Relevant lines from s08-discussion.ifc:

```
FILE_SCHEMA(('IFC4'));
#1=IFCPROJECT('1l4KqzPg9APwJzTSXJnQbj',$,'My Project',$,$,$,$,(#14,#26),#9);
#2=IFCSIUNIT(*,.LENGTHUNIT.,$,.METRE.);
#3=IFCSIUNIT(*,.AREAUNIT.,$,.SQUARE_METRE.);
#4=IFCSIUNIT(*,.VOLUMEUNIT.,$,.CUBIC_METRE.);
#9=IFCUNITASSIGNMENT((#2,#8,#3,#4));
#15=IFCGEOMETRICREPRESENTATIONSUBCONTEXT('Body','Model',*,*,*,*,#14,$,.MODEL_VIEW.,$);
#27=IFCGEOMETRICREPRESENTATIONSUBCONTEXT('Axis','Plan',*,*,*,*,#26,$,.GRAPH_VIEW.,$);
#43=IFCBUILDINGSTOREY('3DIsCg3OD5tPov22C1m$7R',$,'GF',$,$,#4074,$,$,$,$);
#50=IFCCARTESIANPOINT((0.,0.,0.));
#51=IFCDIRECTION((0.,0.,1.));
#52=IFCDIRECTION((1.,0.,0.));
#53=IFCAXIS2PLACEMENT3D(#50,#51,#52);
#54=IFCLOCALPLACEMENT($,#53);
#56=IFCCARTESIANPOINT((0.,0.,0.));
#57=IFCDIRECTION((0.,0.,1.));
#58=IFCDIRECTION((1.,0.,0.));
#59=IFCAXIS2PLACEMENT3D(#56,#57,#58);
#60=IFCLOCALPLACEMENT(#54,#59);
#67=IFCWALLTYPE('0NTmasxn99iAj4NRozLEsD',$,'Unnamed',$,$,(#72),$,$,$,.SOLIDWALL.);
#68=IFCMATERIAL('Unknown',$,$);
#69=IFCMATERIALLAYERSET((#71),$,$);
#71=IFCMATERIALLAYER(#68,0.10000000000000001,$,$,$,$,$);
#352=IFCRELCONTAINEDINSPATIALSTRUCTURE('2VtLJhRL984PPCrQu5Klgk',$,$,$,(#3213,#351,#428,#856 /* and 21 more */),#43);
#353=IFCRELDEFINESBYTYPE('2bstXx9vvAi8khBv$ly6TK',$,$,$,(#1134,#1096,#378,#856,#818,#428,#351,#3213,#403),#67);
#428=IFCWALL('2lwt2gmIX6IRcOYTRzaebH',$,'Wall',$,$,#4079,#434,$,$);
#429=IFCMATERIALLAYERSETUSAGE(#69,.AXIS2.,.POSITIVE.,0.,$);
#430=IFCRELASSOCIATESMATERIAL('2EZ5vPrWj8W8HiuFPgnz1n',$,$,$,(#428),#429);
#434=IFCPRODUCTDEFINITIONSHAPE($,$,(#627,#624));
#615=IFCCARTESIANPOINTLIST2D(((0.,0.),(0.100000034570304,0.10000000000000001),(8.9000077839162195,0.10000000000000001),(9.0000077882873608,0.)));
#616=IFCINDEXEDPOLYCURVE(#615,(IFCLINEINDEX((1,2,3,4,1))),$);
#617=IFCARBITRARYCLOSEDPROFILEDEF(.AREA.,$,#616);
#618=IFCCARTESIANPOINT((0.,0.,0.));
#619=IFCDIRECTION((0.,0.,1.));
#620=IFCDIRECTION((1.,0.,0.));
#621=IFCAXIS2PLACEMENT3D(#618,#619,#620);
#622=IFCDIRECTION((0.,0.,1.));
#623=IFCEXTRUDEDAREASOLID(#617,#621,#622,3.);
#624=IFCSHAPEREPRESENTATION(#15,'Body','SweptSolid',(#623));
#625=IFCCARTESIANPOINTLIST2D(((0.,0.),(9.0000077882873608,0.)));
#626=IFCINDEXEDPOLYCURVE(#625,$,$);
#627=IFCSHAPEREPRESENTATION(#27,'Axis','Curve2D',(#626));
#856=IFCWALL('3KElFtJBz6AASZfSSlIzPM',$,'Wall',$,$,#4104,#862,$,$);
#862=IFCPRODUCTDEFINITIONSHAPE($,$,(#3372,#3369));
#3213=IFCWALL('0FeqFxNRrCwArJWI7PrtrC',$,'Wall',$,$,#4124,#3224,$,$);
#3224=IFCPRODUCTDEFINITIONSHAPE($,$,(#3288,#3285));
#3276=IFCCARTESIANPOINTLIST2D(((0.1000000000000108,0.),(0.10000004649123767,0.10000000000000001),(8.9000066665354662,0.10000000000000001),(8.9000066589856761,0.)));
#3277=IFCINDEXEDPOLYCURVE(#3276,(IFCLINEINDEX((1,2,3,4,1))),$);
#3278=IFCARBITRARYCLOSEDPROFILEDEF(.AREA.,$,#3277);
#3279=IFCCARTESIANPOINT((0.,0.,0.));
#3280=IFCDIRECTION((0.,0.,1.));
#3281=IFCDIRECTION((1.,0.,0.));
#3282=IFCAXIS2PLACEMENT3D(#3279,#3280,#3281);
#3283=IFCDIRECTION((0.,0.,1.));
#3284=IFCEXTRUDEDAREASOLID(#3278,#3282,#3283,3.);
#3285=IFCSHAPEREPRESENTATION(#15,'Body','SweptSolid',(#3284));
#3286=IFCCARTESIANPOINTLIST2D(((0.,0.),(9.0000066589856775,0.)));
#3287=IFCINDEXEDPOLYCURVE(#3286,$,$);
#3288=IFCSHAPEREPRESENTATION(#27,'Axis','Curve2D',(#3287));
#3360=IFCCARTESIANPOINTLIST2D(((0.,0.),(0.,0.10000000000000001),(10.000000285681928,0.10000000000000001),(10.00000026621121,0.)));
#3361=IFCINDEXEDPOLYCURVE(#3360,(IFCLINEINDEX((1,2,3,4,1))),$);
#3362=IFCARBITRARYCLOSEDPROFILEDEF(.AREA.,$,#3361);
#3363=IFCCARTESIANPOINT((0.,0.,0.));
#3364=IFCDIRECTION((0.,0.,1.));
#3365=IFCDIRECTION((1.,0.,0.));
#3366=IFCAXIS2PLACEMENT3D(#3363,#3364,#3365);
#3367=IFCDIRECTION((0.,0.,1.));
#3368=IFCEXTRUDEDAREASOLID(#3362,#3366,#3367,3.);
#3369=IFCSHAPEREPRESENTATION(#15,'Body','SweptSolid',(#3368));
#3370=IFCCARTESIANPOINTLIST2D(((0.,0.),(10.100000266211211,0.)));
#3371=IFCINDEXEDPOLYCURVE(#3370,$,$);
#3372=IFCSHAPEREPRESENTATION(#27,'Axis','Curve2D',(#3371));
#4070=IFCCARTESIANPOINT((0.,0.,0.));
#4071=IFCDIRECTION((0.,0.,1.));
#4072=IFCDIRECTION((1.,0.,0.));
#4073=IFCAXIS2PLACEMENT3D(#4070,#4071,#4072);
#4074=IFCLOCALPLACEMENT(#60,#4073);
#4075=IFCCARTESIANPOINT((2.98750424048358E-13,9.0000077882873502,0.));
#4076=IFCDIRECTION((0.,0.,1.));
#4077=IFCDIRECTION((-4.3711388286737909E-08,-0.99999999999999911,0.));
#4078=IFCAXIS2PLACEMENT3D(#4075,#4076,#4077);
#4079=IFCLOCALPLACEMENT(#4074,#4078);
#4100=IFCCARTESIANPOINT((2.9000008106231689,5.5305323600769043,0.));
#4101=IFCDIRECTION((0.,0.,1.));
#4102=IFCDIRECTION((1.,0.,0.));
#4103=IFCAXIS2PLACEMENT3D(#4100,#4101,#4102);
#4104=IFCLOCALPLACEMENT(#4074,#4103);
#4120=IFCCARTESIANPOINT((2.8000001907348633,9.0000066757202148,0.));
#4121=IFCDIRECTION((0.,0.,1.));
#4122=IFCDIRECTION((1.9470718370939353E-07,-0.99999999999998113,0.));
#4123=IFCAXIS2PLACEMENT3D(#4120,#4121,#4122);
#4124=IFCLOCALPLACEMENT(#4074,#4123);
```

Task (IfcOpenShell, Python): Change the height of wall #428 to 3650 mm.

```python
import ifcopenshell
import ifcopenshell.geom
import ifcopenshell.util.representation
import ifcopenshell.util.shape
import ifcopenshell.util.unit

model = ifcopenshell.open("s08-discussion.ifc")
unit_scale = ifcopenshell.util.unit.calculate_unit_scale(model)
settings = ifcopenshell.geom.settings()


def volume(element):
    """Net volume in cubic metres, openings subtracted."""
    shape = ifcopenshell.geom.create_shape(settings, element)
    return ifcopenshell.util.shape.get_volume(shape.geometry)


wall = model.by_guid("2lwt2gmIX6IRcOYTRzaebH")
before = volume(wall)

body = ifcopenshell.util.representation.get_representation(wall, "Model", "Body")
solid = body.Items[0]
old_height = solid.Depth
solid.Depth = 3.65 / unit_scale
after = volume(wall)

print(f"height {old_height:g} -> {solid.Depth:g}, volume {before:.3f} -> {after:.3f} m3")

model.write("s08-discussion_updated.ifc")
```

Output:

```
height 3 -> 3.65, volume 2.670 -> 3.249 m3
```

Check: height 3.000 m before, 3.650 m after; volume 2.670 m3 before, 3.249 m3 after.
